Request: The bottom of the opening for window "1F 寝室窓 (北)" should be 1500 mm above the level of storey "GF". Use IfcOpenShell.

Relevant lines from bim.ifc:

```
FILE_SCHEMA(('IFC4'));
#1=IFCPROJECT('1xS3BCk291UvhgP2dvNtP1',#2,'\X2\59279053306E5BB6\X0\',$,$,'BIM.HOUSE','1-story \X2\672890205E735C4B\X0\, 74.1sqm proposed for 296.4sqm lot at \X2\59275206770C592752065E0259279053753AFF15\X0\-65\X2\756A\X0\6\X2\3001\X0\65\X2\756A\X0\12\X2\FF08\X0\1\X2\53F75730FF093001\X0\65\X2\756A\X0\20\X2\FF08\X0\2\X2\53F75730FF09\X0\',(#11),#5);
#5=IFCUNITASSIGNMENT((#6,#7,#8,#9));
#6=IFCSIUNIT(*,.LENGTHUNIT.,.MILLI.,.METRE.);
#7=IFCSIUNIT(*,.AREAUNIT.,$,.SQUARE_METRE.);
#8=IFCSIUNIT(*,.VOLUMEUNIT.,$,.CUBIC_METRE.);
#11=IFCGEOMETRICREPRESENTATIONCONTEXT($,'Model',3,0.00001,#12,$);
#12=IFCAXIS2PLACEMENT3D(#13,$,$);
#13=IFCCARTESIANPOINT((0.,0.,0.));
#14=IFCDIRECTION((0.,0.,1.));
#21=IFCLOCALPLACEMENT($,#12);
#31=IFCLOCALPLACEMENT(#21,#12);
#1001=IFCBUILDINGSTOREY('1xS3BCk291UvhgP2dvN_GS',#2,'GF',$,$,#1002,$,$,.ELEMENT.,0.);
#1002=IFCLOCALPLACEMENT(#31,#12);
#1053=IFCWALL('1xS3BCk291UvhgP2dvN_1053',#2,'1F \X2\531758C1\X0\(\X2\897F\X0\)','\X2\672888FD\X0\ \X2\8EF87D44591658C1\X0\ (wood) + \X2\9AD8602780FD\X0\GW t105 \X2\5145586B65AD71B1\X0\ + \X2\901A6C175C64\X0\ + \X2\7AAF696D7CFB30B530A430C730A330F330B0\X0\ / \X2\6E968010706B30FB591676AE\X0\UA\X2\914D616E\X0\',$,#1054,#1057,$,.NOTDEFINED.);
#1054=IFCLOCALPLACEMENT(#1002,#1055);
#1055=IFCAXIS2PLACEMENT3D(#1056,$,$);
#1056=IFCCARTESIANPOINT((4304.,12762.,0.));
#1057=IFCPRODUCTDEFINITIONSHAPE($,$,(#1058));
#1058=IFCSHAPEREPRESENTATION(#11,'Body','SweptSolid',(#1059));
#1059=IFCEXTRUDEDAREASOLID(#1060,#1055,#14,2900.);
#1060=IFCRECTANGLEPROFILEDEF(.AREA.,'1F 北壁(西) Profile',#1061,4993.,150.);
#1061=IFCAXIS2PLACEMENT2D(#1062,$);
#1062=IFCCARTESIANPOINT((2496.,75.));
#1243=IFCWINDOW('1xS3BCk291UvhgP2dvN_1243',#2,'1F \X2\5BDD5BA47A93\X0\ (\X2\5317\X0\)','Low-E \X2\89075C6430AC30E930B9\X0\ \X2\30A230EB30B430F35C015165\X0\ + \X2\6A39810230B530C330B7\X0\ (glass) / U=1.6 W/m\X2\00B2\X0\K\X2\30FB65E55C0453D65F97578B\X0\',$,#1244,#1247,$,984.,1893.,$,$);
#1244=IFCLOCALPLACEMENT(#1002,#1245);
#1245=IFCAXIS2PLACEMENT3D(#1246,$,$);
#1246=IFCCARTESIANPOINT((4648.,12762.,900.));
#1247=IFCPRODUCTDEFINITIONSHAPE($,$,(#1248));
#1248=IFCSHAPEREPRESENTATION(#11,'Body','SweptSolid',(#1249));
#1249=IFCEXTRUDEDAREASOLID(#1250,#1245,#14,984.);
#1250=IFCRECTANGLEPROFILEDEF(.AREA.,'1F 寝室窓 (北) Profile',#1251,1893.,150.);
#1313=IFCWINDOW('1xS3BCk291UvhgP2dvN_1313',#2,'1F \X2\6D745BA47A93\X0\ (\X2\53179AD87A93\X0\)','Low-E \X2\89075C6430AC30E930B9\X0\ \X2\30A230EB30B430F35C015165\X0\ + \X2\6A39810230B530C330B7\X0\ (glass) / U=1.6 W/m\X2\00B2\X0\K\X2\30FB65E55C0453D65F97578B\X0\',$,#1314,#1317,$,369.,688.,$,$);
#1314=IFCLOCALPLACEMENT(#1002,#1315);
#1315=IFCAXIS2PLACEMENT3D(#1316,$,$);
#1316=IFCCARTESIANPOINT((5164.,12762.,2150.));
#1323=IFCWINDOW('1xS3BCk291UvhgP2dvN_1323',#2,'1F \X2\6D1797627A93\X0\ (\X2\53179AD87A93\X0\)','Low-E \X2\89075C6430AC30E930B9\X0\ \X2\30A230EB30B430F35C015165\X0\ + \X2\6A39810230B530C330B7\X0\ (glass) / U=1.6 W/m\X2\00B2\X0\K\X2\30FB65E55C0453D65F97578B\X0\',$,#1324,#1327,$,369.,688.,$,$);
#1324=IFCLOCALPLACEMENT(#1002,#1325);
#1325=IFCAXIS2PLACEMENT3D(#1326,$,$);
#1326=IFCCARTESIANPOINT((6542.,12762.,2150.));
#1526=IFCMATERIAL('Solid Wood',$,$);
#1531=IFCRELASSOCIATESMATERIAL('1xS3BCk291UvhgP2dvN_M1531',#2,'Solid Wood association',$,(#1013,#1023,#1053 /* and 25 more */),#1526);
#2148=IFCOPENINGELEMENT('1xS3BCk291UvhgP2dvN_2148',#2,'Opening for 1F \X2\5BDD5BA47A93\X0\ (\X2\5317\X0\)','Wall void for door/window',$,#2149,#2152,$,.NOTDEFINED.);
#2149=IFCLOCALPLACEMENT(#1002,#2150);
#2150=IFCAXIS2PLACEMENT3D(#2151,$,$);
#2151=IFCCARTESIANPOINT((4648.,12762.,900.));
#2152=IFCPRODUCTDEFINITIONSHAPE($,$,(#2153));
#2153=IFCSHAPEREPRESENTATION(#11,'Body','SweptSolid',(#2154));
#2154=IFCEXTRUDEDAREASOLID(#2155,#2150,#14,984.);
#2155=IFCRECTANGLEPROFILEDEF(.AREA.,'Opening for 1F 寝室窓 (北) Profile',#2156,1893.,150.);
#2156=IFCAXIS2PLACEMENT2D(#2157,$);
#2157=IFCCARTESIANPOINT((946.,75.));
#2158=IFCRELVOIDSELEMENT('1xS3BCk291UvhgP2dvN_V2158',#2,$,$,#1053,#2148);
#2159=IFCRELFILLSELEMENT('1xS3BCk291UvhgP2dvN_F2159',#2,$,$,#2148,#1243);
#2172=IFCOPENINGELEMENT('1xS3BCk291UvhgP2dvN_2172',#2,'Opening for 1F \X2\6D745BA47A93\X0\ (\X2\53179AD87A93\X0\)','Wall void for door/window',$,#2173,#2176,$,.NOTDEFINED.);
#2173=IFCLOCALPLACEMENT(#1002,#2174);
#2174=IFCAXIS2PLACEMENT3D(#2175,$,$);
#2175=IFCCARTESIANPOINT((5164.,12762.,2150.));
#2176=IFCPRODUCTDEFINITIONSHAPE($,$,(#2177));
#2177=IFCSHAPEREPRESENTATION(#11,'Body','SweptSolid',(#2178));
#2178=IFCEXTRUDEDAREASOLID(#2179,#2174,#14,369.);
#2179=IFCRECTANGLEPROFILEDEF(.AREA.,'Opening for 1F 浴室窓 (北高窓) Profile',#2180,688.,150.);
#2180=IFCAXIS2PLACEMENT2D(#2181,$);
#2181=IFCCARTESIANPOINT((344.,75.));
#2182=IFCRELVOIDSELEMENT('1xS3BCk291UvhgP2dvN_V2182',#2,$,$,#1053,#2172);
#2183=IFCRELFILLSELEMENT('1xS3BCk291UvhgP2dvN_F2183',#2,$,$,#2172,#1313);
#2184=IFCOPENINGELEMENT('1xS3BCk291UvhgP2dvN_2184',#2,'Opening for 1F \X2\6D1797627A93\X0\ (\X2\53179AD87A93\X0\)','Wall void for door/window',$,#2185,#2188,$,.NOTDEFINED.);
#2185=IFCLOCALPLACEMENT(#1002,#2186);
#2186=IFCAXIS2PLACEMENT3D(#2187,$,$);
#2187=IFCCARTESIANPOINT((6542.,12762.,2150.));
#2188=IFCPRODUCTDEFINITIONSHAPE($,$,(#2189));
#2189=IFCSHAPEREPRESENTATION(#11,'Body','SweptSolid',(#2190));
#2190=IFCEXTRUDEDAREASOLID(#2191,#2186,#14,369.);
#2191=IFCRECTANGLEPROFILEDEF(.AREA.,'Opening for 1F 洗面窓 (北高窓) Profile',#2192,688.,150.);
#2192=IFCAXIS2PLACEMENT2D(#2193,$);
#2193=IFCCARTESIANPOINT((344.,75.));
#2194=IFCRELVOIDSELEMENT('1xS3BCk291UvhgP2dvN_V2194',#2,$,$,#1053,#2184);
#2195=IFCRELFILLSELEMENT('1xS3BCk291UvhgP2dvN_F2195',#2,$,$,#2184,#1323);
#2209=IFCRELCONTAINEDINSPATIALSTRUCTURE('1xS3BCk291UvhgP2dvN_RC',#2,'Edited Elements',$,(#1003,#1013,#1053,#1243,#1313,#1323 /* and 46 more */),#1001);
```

```python
import numpy as np
import ifcopenshell
import ifcopenshell.api.geometry
import ifcopenshell.geom
import ifcopenshell.util.element
import ifcopenshell.util.placement
import ifcopenshell.util.shape
import ifcopenshell.util.unit

model = ifcopenshell.open("bim.ifc")
unit_scale = ifcopenshell.util.unit.calculate_unit_scale(model)

window = model.by_guid("1xS3BCk291UvhgP2dvN_1243")
opening = window.FillsVoids[0].RelatingOpeningElement
storey = ifcopenshell.util.element.get_container(window, ifc_class="IfcBuildingStorey")
level = ifcopenshell.util.placement.get_local_placement(storey.ObjectPlacement)[2, 3]

# The opening's origin need not be at the sill, so measure its lowest point.
shape = ifcopenshell.geom.create_shape(ifcopenshell.geom.settings(), opening)
bottom = ifcopenshell.util.shape.get_shape_bottom_elevation(shape, shape.geometry) / unit_scale
dz = level + 1500.0 - bottom

shift = np.array([0.0, 0.0, dz])
# The window is not placed relative to its opening, so move both.
for product in (opening, window):
    matrix = ifcopenshell.util.placement.get_local_placement(product.ObjectPlacement)
    matrix[:3, 3] += shift
    ifcopenshell.api.geometry.edit_object_placement(model, product=product, matrix=matrix, is_si=False)

print(f"moved by {dz * unit_scale:+.3f} m")

model.write("bim_v2.ifc")
```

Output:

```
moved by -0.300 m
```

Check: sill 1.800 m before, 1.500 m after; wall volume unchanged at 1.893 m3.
